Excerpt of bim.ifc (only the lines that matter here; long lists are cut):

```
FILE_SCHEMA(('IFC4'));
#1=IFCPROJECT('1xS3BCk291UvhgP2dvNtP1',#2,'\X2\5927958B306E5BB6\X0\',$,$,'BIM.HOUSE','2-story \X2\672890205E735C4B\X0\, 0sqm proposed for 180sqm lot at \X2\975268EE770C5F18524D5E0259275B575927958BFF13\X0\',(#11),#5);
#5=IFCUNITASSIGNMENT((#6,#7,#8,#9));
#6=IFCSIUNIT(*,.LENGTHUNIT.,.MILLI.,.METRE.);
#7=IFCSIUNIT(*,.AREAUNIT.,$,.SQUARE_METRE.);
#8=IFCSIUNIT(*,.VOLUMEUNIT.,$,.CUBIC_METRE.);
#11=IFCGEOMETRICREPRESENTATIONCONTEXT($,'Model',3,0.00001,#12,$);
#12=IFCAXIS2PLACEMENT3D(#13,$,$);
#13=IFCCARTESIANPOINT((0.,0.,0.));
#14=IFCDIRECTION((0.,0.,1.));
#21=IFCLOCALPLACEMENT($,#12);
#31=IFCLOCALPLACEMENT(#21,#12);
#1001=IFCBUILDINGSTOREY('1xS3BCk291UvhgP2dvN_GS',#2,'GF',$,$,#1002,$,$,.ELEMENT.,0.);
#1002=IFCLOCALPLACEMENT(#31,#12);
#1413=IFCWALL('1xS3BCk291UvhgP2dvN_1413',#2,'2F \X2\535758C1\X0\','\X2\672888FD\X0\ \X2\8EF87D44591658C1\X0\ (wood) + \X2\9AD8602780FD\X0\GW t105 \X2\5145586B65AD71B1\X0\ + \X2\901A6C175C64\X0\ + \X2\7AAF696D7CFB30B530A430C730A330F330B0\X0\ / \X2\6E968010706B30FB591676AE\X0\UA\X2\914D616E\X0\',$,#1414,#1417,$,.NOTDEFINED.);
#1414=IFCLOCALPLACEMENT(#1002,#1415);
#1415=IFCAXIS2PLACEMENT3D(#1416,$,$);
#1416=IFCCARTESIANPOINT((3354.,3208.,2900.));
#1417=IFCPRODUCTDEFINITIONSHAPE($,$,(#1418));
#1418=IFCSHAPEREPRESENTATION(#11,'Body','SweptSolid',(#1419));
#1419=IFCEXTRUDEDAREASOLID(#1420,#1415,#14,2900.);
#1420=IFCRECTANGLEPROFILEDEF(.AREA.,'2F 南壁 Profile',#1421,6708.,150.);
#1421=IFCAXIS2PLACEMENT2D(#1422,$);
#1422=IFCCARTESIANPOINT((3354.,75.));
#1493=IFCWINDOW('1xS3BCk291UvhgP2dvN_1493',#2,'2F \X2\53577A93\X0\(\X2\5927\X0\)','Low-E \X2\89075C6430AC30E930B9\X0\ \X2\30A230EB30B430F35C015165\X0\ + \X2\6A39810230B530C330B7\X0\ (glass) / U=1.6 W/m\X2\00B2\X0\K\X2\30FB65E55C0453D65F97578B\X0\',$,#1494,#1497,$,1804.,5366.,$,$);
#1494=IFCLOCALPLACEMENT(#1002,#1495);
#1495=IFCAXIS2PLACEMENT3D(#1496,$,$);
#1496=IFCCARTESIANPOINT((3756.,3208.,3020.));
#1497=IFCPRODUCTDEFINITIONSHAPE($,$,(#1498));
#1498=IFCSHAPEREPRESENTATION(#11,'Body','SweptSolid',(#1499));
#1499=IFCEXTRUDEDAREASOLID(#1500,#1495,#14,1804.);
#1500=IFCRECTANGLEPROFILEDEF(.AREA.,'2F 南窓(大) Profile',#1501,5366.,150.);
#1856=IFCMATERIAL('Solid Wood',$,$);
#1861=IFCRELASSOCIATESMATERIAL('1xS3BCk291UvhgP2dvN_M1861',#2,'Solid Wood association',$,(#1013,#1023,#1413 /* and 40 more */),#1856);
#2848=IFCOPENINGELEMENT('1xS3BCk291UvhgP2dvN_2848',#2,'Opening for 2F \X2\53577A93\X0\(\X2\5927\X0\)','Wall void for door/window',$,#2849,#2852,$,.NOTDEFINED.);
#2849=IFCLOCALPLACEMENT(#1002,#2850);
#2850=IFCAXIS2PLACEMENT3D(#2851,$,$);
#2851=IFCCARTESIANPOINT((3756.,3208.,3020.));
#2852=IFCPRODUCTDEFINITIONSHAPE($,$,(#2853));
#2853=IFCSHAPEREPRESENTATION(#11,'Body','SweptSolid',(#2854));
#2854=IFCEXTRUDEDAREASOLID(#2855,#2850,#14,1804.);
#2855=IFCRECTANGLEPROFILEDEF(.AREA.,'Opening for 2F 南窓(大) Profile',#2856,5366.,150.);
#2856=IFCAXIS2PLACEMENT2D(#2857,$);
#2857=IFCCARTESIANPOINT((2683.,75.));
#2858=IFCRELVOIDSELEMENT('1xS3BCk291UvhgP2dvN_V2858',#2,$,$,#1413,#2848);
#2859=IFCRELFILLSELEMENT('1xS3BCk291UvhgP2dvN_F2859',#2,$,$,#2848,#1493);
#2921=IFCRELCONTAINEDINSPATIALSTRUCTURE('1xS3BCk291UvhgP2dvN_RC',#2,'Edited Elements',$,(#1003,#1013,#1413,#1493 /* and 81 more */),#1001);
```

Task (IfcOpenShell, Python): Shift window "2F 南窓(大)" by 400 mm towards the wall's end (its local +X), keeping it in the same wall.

```python
import ifcopenshell
import ifcopenshell.api.geometry
import ifcopenshell.util.placement
import ifcopenshell.util.unit

model = ifcopenshell.open("bim.ifc")
unit_scale = ifcopenshell.util.unit.calculate_unit_scale(model)

window = model.by_guid("1xS3BCk291UvhgP2dvN_1493")
opening = window.FillsVoids[0].RelatingOpeningElement
wall = opening.VoidsElements[0].RelatingBuildingElement

wall_matrix = ifcopenshell.util.placement.get_local_placement(wall.ObjectPlacement)
shift = wall_matrix[:3, 0] * 0.4 / unit_scale
before = ifcopenshell.util.placement.get_local_placement(window.ObjectPlacement)[:3, 3].copy()

# The window is not placed relative to its opening, so move both.
for product in (opening, window):
    matrix = ifcopenshell.util.placement.get_local_placement(product.ObjectPlacement)
    matrix[:3, 3] += shift
    ifcopenshell.api.geometry.edit_object_placement(model, product=product, matrix=matrix, is_si=False)

after = ifcopenshell.util.placement.get_local_placement(window.ObjectPlacement)[:3, 3]
print("window moved by", (after - before).round(3) + 0.0)

model.write("bim_rev.ifc")
```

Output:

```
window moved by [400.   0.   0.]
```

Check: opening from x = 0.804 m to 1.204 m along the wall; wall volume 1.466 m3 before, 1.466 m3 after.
